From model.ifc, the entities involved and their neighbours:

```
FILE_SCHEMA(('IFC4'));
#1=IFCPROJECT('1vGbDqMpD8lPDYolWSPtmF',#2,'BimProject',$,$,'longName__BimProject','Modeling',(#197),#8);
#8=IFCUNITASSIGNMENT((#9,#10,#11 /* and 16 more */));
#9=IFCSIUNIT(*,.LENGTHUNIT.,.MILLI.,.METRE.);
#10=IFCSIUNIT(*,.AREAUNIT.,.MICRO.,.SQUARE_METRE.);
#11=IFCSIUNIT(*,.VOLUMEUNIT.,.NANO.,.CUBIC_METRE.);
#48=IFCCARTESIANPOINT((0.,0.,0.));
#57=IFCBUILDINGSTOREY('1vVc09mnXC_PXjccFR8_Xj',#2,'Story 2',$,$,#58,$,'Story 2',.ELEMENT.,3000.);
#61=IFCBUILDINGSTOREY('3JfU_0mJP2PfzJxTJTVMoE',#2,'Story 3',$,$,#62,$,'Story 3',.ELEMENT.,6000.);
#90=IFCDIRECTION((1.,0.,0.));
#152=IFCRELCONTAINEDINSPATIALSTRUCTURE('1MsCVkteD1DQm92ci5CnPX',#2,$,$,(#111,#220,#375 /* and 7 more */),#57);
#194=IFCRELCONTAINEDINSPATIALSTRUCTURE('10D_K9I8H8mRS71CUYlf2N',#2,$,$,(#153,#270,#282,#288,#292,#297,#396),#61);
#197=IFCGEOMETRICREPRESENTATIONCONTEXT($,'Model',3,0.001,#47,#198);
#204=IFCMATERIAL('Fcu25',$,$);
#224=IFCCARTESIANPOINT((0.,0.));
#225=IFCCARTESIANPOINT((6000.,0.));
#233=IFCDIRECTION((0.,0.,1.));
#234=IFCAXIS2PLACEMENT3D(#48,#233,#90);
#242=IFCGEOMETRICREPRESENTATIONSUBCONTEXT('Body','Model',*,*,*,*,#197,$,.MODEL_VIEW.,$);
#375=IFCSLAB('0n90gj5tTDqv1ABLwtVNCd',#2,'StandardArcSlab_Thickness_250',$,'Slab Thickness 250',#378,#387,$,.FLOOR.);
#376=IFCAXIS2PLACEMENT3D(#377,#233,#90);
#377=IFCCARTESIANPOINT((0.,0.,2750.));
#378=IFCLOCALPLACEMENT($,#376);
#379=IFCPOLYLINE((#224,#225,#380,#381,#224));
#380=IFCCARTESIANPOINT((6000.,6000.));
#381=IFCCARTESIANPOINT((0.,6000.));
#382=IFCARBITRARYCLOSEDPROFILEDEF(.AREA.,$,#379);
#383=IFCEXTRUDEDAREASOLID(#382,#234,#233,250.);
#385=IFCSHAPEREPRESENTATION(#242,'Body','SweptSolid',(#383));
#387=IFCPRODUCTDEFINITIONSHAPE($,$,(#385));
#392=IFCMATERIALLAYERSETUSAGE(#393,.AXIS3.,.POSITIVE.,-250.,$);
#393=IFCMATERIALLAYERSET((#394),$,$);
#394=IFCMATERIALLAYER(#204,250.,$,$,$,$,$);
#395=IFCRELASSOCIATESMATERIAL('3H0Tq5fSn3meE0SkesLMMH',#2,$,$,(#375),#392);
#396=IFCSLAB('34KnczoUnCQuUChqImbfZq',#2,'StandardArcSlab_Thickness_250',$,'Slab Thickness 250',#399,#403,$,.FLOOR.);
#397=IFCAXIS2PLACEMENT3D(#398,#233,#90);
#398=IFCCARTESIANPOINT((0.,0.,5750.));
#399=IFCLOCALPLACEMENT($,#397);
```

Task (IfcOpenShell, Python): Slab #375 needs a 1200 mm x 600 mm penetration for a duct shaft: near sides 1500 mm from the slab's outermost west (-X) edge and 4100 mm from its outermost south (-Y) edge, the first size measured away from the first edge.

```python
import numpy as np
import ifcopenshell
import ifcopenshell.api.feature
import ifcopenshell.api.geometry
import ifcopenshell.api.root
import ifcopenshell.geom
import ifcopenshell.util.placement
import ifcopenshell.util.representation
import ifcopenshell.util.shape
import ifcopenshell.util.unit

model = ifcopenshell.open("model.ifc")
unit_scale = ifcopenshell.util.unit.calculate_unit_scale(model)
settings = ifcopenshell.geom.settings()


def volume(element):
    """Net volume in cubic metres, openings subtracted."""
    shape = ifcopenshell.geom.create_shape(settings, element)
    return ifcopenshell.util.shape.get_volume(shape.geometry)


slab = model.by_guid("0n90gj5tTDqv1ABLwtVNCd")
before = volume(slab)

# Extent in the slab's own axes, in metres. The edges named are its -X and -Y sides.
slab_shape = ifcopenshell.geom.create_shape(settings, slab)
vertices = ifcopenshell.util.shape.get_vertices(slab_shape.geometry)
x_min, y_min, bottom = vertices.min(axis=0)
top = vertices[:, 2].max()

opening = ifcopenshell.api.root.create_entity(model, ifc_class="IfcOpeningElement", name="Duct shaft opening", predefined_type="OPENING")
context = ifcopenshell.util.representation.get_context(model, "Model", "Body", "MODEL_VIEW")
width, depth = 1.2, 0.6
outline = [(0.0, 0.0), (width, 0.0), (width, depth), (0.0, depth), (0.0, 0.0)]
# Overshoot both faces by 50 mm so the cut is clean.
shape = ifcopenshell.api.geometry.add_slab_representation(
    model, context=context, depth=top - bottom + 0.1, polyline=outline
)
ifcopenshell.api.geometry.assign_representation(model, product=opening, representation=shape)

matrix = ifcopenshell.util.placement.get_local_placement(slab.ObjectPlacement)
matrix[:, 3] = matrix @ np.append(np.array([x_min + 1.5, y_min + 4.1, bottom - 0.05]) / unit_scale, 1.0)
ifcopenshell.api.geometry.edit_object_placement(model, product=opening, matrix=matrix, is_si=False)
ifcopenshell.api.feature.add_feature(model, feature=opening, element=slab)

after = volume(slab)

print(f"slab volume {before:.3f} -> {after:.3f} m3")

model.write("model_updated.ifc")
```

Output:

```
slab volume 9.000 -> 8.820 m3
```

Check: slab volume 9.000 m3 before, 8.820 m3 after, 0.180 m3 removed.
